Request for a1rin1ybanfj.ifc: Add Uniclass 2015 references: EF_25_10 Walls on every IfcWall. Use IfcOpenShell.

First a look at what the model holds.

```python
import ifcopenshell

model = ifcopenshell.open("a1rin1ybanfj.ifc")
print(model.schema)
print("classifications:", [c.Name for c in model.by_type("IfcClassification")])
for ifc_class in ("IfcDoor", "IfcRoof", "IfcStair", "IfcWall", "IfcWindow"):
    print(ifc_class, len(model.by_type(ifc_class)))
```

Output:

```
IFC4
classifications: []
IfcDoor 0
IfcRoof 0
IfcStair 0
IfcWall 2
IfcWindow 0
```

```python
import ifcopenshell
import ifcopenshell.api.classification

model = ifcopenshell.open("a1rin1ybanfj.ifc")

system = ifcopenshell.api.classification.add_classification(model, classification="Uniclass 2015")

codes = {
    "IfcWall": ("EF_25_10", "Walls"),
}
for ifc_class, (code, name) in codes.items():
    products = model.by_type(ifc_class)
    ifcopenshell.api.classification.add_reference(
        model, products=products, classification=system, identification=code, name=name
    )
    print(code, len(products))

model.write("a1rin1ybanfj_edited.ifc")
```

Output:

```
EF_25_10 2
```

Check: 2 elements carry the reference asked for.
